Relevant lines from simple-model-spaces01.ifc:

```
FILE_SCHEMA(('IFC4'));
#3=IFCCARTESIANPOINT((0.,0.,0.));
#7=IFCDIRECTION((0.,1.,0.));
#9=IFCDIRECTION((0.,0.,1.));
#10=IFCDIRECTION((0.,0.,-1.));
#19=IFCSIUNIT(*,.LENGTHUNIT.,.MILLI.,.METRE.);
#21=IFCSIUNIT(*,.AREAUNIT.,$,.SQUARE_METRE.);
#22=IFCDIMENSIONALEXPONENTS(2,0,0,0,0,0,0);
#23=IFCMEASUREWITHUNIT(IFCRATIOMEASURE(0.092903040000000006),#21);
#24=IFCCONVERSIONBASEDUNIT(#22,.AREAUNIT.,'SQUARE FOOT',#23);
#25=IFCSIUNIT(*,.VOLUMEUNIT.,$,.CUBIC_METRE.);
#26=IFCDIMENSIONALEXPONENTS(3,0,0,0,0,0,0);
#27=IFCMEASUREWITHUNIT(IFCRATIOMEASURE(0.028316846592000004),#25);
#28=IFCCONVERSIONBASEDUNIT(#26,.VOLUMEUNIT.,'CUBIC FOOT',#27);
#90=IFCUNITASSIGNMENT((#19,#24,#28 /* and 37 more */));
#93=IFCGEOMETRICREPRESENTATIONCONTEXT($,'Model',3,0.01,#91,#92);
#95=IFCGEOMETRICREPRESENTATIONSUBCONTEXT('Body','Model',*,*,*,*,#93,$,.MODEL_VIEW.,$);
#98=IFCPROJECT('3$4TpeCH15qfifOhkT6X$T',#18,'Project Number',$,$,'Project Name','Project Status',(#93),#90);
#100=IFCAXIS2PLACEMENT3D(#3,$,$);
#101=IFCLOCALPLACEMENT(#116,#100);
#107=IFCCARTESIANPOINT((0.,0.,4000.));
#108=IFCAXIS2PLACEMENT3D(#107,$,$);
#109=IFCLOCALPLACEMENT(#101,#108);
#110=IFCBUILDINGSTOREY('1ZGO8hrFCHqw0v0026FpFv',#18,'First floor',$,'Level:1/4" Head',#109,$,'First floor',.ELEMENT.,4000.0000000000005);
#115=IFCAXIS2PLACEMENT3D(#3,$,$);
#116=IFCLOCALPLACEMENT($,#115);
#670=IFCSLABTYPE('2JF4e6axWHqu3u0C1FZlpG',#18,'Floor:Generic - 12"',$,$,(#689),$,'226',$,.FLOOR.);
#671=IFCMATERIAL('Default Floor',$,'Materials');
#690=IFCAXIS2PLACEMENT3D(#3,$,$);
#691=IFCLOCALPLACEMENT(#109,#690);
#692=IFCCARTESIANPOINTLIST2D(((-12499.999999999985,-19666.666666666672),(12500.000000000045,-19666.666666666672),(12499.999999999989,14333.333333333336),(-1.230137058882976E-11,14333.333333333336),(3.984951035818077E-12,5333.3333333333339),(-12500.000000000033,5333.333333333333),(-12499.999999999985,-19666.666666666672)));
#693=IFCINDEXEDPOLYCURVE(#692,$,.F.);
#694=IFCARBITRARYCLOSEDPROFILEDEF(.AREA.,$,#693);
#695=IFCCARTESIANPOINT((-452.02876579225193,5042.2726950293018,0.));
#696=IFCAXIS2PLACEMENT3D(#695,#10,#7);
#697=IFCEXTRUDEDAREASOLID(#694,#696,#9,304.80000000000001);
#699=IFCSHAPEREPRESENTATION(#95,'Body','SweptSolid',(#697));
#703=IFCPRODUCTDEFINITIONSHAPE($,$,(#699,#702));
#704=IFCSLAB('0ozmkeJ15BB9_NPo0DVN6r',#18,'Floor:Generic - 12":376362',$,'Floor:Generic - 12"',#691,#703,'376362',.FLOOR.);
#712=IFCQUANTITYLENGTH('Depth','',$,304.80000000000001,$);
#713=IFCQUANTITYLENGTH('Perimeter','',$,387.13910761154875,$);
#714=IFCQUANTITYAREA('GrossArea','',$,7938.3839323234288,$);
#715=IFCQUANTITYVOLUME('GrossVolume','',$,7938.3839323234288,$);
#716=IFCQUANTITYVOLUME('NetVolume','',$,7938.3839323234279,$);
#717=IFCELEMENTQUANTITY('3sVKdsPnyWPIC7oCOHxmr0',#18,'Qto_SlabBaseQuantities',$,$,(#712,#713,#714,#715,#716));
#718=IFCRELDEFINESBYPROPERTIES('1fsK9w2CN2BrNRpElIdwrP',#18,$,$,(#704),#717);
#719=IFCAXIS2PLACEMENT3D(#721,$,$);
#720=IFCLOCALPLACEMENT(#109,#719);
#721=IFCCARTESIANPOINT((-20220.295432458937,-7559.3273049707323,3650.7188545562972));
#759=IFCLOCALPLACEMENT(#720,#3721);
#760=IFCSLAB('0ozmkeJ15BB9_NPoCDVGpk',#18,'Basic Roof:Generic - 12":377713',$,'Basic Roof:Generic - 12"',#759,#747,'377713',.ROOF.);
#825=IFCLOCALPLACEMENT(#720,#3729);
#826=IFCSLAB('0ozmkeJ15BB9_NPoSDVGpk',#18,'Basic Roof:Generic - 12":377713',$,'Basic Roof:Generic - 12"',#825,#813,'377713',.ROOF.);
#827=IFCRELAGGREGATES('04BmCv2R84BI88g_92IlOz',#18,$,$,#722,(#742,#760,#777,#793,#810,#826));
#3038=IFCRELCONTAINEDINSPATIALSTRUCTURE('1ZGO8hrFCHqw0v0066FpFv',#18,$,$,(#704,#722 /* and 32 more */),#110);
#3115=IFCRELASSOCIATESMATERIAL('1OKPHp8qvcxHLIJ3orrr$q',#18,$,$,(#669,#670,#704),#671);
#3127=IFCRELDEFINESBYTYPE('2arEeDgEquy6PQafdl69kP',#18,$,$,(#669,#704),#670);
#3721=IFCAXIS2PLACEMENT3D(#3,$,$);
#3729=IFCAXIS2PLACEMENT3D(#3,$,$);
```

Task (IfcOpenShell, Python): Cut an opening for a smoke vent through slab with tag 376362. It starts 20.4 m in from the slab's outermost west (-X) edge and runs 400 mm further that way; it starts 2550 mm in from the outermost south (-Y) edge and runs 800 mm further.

```python
import numpy as np
import ifcopenshell
import ifcopenshell.api.feature
import ifcopenshell.api.geometry
import ifcopenshell.api.pset
import ifcopenshell.api.root
import ifcopenshell.geom
import ifcopenshell.util.element
import ifcopenshell.util.placement
import ifcopenshell.util.representation
import ifcopenshell.util.shape
import ifcopenshell.util.unit

model = ifcopenshell.open("simple-model-spaces01.ifc")
unit_scale = ifcopenshell.util.unit.calculate_unit_scale(model)
volume_scale = ifcopenshell.util.unit.calculate_unit_scale(model, "VOLUMEUNIT")
settings = ifcopenshell.geom.settings()


def volume(element):
    """Net volume in cubic metres, openings subtracted."""
    shape = ifcopenshell.geom.create_shape(settings, element)
    return ifcopenshell.util.shape.get_volume(shape.geometry)


slab = model.by_guid("0ozmkeJ15BB9_NPo0DVN6r")
before = volume(slab)

# Extent in the slab's own axes, in metres. The edges named are its -X and -Y sides.
slab_shape = ifcopenshell.geom.create_shape(settings, slab)
vertices = ifcopenshell.util.shape.get_vertices(slab_shape.geometry)
x_min, y_min, bottom = vertices.min(axis=0)
top = vertices[:, 2].max()

opening = ifcopenshell.api.root.create_entity(model, ifc_class="IfcOpeningElement", name="Smoke vent opening", predefined_type="OPENING")
context = ifcopenshell.util.representation.get_context(model, "Model", "Body", "MODEL_VIEW")
width, depth = 0.4, 0.8
outline = [(0.0, 0.0), (width, 0.0), (width, depth), (0.0, depth), (0.0, 0.0)]
# Overshoot both faces by 50 mm so the cut is clean.
shape = ifcopenshell.api.geometry.add_slab_representation(
    model, context=context, depth=top - bottom + 0.1, polyline=outline
)
ifcopenshell.api.geometry.assign_representation(model, product=opening, representation=shape)

matrix = ifcopenshell.util.placement.get_local_placement(slab.ObjectPlacement)
matrix[:, 3] = matrix @ np.append(np.array([x_min + 20.4, y_min + 2.55, bottom - 0.05]) / unit_scale, 1.0)
ifcopenshell.api.geometry.edit_object_placement(model, product=opening, matrix=matrix, is_si=False)
ifcopenshell.api.feature.add_feature(model, feature=opening, element=slab)

after = volume(slab)

# Update the slab's stored quantities.
qto = model.by_id(ifcopenshell.util.element.get_pset(slab, "Qto_SlabBaseQuantities", should_inherit=False)["id"])
ifcopenshell.api.pset.edit_qto(model, qto=qto, properties={"NetVolume": after / volume_scale})

print(f"slab volume {before:.3f} -> {after:.3f} m3")

model.write("simple-model-spaces01_v2.ifc")
```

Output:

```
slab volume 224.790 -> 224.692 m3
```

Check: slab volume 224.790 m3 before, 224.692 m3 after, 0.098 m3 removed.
